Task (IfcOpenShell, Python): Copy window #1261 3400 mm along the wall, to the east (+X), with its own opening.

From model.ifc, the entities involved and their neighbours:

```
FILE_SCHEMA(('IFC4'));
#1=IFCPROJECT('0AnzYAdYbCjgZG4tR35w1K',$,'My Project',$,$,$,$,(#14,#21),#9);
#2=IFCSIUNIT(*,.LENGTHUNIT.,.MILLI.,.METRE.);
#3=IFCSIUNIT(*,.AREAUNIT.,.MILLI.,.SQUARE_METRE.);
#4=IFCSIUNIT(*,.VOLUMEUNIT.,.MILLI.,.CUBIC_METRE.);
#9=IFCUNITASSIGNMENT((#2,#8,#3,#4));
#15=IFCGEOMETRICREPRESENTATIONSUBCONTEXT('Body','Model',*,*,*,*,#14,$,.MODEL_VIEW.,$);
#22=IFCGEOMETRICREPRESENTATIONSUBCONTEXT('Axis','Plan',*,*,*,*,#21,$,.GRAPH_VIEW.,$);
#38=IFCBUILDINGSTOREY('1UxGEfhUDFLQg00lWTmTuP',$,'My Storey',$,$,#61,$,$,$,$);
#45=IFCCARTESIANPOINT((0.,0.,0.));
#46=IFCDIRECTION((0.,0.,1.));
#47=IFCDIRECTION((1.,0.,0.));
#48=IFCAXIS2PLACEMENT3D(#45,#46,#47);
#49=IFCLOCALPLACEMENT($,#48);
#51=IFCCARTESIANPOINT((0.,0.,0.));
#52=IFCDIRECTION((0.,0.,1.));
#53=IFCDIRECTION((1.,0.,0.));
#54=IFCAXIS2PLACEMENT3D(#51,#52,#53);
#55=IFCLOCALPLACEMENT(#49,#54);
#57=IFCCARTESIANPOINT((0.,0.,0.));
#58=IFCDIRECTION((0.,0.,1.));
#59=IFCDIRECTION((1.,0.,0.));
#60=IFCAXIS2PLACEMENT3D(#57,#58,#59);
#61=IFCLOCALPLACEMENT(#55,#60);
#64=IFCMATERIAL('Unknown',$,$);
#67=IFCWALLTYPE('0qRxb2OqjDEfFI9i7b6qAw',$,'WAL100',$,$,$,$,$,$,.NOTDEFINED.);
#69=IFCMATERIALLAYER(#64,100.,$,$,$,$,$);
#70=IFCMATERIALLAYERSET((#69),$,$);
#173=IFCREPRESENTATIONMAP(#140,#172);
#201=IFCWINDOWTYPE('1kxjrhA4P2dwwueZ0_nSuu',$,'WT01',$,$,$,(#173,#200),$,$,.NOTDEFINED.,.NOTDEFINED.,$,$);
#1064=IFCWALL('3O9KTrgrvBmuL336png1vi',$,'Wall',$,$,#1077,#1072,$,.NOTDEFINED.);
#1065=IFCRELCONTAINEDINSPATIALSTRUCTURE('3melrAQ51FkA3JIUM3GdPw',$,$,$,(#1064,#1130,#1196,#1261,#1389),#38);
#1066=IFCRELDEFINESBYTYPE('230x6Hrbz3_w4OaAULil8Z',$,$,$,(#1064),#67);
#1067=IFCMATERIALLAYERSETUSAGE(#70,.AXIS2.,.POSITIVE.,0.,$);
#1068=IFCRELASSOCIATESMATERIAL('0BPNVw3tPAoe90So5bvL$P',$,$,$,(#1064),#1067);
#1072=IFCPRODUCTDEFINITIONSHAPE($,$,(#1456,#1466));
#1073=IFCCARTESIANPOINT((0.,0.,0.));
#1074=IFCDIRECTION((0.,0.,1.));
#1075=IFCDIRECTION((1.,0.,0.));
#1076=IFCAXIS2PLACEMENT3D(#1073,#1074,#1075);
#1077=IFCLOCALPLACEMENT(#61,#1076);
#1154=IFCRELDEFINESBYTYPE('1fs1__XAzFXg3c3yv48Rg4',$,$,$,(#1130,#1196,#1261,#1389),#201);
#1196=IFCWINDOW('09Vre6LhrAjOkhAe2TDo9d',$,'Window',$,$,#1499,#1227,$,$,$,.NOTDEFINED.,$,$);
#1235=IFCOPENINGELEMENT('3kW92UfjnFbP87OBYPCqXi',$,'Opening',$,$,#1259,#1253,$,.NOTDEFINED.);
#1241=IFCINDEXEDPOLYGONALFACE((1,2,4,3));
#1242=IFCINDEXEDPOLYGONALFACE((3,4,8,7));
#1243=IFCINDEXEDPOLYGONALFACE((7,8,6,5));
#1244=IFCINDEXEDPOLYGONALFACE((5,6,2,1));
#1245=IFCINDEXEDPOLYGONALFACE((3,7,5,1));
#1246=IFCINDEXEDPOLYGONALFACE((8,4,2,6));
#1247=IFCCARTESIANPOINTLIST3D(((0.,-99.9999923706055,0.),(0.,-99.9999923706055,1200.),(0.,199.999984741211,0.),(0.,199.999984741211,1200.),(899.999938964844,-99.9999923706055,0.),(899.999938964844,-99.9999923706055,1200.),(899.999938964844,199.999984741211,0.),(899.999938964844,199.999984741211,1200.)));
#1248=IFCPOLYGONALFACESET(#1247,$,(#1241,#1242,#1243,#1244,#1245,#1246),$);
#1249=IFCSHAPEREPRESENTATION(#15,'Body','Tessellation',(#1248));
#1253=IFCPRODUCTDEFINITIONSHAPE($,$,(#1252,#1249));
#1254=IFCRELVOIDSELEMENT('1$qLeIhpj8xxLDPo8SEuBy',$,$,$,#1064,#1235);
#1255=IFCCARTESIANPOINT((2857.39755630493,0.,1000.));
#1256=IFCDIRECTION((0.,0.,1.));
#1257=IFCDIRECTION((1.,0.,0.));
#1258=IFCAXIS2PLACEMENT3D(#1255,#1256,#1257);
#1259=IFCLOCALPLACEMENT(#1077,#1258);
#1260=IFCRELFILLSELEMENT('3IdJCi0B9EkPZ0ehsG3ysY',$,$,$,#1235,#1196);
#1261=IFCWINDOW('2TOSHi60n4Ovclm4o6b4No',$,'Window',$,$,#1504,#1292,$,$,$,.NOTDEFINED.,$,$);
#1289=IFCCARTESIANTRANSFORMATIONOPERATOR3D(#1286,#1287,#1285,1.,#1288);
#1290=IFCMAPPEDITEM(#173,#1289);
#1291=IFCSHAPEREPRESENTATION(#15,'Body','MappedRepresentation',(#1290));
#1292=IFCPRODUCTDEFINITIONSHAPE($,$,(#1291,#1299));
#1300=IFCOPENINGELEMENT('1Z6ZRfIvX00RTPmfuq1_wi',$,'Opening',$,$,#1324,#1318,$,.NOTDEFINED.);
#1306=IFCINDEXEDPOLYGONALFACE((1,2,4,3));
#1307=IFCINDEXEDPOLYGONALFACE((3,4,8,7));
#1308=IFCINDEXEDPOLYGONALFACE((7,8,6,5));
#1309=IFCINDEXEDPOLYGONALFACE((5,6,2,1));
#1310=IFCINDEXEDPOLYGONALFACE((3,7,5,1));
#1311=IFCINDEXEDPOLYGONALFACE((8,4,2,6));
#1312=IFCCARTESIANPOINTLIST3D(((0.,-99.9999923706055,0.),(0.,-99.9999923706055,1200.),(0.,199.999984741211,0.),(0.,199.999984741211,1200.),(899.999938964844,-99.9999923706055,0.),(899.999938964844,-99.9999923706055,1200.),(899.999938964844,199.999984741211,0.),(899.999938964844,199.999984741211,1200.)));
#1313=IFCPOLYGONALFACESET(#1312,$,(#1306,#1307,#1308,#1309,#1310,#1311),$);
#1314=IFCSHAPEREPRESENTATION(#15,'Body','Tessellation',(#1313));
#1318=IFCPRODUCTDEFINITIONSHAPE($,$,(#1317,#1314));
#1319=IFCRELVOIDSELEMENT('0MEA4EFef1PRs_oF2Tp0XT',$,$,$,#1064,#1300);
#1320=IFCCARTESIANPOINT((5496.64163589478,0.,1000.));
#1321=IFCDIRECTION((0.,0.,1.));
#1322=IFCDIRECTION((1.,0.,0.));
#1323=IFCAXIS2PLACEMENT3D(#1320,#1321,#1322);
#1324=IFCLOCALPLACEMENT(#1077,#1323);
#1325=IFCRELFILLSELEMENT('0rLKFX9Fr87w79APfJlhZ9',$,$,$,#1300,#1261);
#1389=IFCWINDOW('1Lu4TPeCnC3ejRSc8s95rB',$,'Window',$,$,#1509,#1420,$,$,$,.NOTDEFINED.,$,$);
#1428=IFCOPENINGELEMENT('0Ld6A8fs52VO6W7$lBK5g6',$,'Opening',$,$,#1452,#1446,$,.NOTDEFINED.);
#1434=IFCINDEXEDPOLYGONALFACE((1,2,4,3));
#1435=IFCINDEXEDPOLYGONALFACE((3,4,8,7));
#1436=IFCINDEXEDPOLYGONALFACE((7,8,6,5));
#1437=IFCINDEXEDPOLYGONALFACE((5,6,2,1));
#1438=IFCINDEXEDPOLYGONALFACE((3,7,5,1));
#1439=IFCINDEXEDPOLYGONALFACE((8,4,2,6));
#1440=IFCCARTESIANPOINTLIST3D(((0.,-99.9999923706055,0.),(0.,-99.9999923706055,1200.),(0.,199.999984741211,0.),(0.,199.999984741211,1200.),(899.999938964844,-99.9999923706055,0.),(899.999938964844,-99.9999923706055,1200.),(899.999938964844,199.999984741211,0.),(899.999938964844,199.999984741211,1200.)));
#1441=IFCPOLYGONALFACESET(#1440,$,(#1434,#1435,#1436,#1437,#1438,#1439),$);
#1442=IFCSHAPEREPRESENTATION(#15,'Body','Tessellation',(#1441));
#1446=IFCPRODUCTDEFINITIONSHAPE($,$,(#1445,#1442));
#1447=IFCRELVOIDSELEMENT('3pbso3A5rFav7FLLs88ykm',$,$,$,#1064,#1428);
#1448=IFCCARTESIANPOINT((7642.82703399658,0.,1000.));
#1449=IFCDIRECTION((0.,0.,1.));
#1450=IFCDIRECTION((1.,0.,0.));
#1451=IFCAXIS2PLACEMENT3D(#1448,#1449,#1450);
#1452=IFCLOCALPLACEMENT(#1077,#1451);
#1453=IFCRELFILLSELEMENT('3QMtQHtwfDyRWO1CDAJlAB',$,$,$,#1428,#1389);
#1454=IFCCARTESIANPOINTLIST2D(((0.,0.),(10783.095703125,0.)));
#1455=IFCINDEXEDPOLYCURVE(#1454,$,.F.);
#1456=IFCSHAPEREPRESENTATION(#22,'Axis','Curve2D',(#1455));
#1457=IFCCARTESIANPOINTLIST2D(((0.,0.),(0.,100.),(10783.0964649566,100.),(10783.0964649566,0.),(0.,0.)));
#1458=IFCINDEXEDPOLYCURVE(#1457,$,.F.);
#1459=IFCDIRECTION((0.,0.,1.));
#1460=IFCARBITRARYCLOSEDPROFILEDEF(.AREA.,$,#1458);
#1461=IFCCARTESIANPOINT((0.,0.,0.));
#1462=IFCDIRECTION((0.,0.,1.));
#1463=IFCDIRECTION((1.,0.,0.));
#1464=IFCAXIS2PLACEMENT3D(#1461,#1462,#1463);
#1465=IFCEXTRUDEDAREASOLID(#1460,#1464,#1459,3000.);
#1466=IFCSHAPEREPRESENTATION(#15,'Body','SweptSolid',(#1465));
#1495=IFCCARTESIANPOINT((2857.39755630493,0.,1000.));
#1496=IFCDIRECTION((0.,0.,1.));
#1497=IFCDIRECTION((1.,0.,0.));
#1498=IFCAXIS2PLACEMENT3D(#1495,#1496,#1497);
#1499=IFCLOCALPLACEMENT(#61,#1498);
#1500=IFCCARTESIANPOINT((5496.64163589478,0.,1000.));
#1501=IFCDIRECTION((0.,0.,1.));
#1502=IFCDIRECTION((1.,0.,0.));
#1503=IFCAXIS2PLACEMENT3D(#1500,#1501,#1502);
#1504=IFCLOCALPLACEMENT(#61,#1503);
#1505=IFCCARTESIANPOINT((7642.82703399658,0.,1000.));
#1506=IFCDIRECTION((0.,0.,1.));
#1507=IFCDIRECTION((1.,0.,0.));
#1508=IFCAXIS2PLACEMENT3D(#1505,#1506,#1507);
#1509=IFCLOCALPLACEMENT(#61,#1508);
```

```python
import ifcopenshell
import ifcopenshell.api.feature
import ifcopenshell.api.geometry
import ifcopenshell.api.root
import ifcopenshell.geom
import ifcopenshell.util.element
import ifcopenshell.util.placement
import ifcopenshell.util.shape

model = ifcopenshell.open("model.ifc")
settings = ifcopenshell.geom.settings()


def volume(element):
    """Net volume in cubic metres, openings subtracted."""
    shape = ifcopenshell.geom.create_shape(settings, element)
    return ifcopenshell.util.shape.get_volume(shape.geometry)


window = model.by_id(1261)
opening = window.FillsVoids[0].RelatingOpeningElement
wall = opening.VoidsElements[0].RelatingBuildingElement
before = volume(wall)
shift = ifcopenshell.util.placement.get_local_placement(wall.ObjectPlacement)[:3, 0] * 3400.0

# copy_class copies the void relationship, type, container and properties, but no geometry.
new_opening = ifcopenshell.api.root.copy_class(model, product=opening)
new_opening.Representation = ifcopenshell.util.element.copy_deep(
    model, opening.Representation, exclude=["IfcGeometricRepresentationContext", "IfcRepresentationMap"]
)
new_window = ifcopenshell.api.root.copy_class(model, product=window)
new_window.Representation = ifcopenshell.util.element.copy_deep(
    model, window.Representation, exclude=["IfcGeometricRepresentationContext", "IfcRepresentationMap"]
)
ifcopenshell.api.feature.add_filling(model, opening=new_opening, element=new_window)

for old, new in ((opening, new_opening), (window, new_window)):
    matrix = ifcopenshell.util.placement.get_local_placement(old.ObjectPlacement)
    matrix[:3, 3] += shift
    ifcopenshell.api.geometry.edit_object_placement(model, product=new, matrix=matrix, is_si=False)

after = volume(wall)

print(f"wall volume {before:.3f} -> {after:.3f} m3")

model.write("model_edited.ifc")
```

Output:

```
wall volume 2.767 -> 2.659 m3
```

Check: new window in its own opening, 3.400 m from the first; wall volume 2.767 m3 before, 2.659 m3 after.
